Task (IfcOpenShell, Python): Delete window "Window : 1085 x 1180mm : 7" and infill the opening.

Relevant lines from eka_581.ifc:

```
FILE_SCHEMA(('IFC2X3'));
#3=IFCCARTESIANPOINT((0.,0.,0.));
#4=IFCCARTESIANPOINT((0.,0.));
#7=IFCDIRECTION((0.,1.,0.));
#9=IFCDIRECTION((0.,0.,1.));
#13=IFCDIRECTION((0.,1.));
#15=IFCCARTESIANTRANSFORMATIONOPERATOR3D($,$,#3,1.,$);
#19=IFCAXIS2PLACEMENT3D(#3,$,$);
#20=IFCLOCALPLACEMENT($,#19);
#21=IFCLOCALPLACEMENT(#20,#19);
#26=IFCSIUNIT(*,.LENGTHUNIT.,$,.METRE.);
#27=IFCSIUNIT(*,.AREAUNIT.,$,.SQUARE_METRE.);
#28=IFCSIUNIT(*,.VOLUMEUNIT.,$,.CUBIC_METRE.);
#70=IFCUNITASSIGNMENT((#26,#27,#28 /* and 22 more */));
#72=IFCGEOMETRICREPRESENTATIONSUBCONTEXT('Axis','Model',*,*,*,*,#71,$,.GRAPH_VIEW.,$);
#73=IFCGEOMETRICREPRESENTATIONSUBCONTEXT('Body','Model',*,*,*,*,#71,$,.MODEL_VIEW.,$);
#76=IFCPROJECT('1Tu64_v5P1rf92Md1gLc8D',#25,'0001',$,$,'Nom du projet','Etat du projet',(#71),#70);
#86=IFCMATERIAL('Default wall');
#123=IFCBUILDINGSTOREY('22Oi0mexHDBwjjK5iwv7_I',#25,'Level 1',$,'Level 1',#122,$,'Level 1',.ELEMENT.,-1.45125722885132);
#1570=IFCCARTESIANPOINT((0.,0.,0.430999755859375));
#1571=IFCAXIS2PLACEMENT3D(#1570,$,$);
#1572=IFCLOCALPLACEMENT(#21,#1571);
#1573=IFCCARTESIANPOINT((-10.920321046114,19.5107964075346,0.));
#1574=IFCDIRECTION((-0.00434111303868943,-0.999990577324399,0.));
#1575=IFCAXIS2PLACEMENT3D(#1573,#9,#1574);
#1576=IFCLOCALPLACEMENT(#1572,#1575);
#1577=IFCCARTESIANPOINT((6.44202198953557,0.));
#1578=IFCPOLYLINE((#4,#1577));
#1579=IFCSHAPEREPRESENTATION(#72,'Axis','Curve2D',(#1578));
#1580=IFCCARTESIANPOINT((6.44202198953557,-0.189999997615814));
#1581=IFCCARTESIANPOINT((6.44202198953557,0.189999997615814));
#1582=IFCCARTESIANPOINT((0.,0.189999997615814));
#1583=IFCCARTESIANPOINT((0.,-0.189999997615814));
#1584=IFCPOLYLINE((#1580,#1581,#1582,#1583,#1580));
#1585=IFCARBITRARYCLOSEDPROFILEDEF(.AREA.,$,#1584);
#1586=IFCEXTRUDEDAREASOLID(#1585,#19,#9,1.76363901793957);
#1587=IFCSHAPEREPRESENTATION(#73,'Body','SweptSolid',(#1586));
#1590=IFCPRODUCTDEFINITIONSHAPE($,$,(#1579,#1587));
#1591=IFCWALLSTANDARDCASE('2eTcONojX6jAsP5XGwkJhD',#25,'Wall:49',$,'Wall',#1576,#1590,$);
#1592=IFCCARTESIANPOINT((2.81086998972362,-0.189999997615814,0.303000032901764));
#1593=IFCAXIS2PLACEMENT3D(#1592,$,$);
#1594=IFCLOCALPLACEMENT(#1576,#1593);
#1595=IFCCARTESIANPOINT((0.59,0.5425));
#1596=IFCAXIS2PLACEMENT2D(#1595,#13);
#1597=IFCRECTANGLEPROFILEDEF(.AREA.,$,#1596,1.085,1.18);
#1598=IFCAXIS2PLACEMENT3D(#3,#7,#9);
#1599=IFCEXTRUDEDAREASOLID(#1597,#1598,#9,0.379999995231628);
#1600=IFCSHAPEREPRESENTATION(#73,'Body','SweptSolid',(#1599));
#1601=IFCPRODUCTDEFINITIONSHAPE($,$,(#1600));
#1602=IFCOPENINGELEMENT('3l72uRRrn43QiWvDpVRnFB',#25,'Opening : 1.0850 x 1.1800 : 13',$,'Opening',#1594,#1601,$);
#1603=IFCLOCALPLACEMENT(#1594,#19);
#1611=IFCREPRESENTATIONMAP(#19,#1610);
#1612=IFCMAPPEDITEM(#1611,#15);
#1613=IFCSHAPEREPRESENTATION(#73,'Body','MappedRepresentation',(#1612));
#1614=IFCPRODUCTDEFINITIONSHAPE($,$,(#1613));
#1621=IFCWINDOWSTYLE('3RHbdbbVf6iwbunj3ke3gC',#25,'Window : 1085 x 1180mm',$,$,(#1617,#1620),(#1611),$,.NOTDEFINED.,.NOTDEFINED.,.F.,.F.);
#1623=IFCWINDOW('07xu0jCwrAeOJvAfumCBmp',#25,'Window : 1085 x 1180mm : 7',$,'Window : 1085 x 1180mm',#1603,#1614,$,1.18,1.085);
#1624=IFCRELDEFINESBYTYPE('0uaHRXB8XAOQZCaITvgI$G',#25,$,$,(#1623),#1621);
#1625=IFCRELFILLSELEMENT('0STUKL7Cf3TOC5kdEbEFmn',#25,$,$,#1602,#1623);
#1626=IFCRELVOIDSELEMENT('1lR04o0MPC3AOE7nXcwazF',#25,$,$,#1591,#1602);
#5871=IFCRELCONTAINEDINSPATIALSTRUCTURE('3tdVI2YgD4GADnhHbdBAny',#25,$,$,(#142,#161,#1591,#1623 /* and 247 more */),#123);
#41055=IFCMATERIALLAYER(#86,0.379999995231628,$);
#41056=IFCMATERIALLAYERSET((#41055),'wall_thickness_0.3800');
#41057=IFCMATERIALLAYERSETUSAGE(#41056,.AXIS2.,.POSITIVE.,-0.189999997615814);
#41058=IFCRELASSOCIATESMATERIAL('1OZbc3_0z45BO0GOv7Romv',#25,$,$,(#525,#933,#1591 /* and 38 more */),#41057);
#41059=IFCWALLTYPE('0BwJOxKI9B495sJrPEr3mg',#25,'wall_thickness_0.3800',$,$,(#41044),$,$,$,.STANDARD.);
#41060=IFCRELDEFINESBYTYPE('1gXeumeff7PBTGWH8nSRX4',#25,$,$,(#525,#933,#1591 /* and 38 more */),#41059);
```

```python
import ifcopenshell
import ifcopenshell.api.feature
import ifcopenshell.api.root
import ifcopenshell.geom
import ifcopenshell.util.shape

model = ifcopenshell.open("eka_581.ifc")
settings = ifcopenshell.geom.settings()


def volume(element):
    """Net volume in cubic metres, openings subtracted."""
    shape = ifcopenshell.geom.create_shape(settings, element)
    return ifcopenshell.util.shape.get_volume(shape.geometry)


window = model.by_guid("07xu0jCwrAeOJvAfumCBmp")
opening = window.FillsVoids[0].RelatingOpeningElement
wall = opening.VoidsElements[0].RelatingBuildingElement
before = volume(wall)

ifcopenshell.api.root.remove_product(model, product=window)
ifcopenshell.api.feature.remove_feature(model, feature=opening)

after = volume(wall)

print(f"wall volume {before:.3f} -> {after:.3f} m3")

model.write("eka_581_updated.ifc")
```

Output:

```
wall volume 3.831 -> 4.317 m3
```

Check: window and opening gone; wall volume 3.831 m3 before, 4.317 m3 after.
